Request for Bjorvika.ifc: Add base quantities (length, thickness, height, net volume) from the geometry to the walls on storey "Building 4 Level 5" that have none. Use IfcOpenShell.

First a look at what the model holds.

```python
import ifcopenshell
import ifcopenshell.util.element
import ifcopenshell.util.unit

model = ifcopenshell.open("Bjorvika.ifc")
print(model.schema)
for unit_type in ("LENGTHUNIT", "AREAUNIT", "VOLUMEUNIT"):
    print(unit_type, ifcopenshell.util.unit.calculate_unit_scale(model, unit_type))
storey = next(s for s in model.by_type("IfcBuildingStorey") if s.Name == "Building 4 Level 5")
walls = [e for e in ifcopenshell.util.element.get_decomposition(storey) if e.is_a("IfcWall")]
for e in sorted(walls, key=lambda e: e.id()):
    print(e.id(), e.is_a(), e.Name, list(ifcopenshell.util.element.get_psets(e, qtos_only=True)), sep=" | ")
```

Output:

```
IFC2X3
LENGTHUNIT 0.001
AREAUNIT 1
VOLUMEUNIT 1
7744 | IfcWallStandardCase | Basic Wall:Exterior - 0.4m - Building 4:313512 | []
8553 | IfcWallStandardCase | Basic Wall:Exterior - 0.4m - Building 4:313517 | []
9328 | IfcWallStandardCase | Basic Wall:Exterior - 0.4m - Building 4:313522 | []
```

```python
import ifcopenshell
import ifcopenshell.api.pset
import ifcopenshell.geom
import ifcopenshell.util.element
import ifcopenshell.util.shape
import ifcopenshell.util.unit

model = ifcopenshell.open("Bjorvika.ifc")
unit_scale = ifcopenshell.util.unit.calculate_unit_scale(model)
volume_scale = ifcopenshell.util.unit.calculate_unit_scale(model, "VOLUMEUNIT")
settings = ifcopenshell.geom.settings()

storey = next(s for s in model.by_type("IfcBuildingStorey") if s.Name == "Building 4 Level 5")
walls = [e for e in ifcopenshell.util.element.get_decomposition(storey) if e.is_a("IfcWall")]

for e in sorted(walls, key=lambda e: e.id()):
    if ifcopenshell.util.element.get_psets(e, qtos_only=True, should_inherit=False):
        continue
    # Geometry comes back in metres, in the element's own axes.
    shape = ifcopenshell.geom.create_shape(settings, e)
    values = {
        "Length": ifcopenshell.util.shape.get_x(shape.geometry) / unit_scale,
        "Width": ifcopenshell.util.shape.get_y(shape.geometry) / unit_scale,
        "Height": ifcopenshell.util.shape.get_z(shape.geometry) / unit_scale,
        "NetVolume": ifcopenshell.util.shape.get_volume(shape.geometry) / volume_scale,
    }
    qto = ifcopenshell.api.pset.add_qto(model, product=e, name="BaseQuantities")
    ifcopenshell.api.pset.edit_qto(model, qto=qto, properties=values)
    print(e.id(), {k: round(v, 3) for k, v in values.items()})

model.write("Bjorvika-out.ifc")
```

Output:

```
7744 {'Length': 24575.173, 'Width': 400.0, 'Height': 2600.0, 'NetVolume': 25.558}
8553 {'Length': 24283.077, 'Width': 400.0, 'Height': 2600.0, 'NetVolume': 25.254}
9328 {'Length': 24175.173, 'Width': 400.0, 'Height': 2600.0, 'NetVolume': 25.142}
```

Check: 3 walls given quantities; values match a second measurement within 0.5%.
